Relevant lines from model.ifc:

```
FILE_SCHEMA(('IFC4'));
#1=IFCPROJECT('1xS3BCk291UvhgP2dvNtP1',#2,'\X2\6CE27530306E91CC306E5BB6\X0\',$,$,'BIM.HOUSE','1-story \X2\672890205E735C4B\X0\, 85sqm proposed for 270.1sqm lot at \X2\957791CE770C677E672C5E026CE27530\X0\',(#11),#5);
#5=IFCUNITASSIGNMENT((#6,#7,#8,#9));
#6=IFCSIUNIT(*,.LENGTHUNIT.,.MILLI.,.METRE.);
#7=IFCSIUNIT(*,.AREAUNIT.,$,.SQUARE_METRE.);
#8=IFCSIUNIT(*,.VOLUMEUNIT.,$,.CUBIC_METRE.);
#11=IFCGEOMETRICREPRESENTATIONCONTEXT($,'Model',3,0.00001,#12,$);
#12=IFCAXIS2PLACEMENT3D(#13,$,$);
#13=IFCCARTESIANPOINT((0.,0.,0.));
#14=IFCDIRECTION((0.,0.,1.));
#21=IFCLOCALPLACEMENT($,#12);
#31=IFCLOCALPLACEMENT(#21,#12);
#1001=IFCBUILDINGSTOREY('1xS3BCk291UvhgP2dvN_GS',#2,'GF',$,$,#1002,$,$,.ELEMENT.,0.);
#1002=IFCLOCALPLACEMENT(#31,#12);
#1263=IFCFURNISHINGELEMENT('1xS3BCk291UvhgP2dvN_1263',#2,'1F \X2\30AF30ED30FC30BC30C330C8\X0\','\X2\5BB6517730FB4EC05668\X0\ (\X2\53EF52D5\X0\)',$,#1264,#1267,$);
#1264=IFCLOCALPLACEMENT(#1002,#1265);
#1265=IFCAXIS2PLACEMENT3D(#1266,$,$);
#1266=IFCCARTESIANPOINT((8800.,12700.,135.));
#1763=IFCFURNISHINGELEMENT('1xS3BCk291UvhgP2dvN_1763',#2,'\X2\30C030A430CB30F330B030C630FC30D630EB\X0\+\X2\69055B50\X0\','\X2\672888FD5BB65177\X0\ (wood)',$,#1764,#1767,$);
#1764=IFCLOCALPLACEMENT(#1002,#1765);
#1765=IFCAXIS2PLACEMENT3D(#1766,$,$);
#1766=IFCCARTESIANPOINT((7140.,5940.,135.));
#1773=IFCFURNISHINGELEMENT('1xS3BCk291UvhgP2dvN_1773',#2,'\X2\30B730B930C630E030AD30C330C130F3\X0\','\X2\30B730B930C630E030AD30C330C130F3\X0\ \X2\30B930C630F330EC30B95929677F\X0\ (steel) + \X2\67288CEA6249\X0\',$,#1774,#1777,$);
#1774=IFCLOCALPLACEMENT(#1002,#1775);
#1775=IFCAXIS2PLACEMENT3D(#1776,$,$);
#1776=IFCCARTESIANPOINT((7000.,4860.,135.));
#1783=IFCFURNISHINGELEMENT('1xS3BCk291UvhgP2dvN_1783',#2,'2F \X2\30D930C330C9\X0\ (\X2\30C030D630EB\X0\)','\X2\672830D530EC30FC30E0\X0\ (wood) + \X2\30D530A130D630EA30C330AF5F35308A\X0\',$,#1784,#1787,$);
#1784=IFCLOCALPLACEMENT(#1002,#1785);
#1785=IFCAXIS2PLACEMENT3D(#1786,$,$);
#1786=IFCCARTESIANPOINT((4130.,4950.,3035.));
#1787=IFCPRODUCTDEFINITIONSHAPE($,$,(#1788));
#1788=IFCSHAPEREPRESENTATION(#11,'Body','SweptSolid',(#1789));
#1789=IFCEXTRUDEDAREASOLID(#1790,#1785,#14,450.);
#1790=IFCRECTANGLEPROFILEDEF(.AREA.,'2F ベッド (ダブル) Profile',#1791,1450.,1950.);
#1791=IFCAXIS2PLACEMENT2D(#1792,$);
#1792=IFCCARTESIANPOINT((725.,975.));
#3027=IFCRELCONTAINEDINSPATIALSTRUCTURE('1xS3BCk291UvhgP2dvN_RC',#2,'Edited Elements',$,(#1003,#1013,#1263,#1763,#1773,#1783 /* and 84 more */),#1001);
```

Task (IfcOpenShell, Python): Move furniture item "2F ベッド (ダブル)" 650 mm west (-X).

```python
import ifcopenshell
import ifcopenshell.api.geometry
import ifcopenshell.util.placement
import ifcopenshell.util.unit

model = ifcopenshell.open("model.ifc")
unit_scale = ifcopenshell.util.unit.calculate_unit_scale(model)

item = model.by_id(1783)
matrix = ifcopenshell.util.placement.get_local_placement(item.ObjectPlacement)
matrix[0, 3] -= 0.65 / unit_scale
ifcopenshell.api.geometry.edit_object_placement(model, product=item, matrix=matrix, is_si=False)

print(ifcopenshell.util.placement.get_local_placement(item.ObjectPlacement).round(3) + 0.0)

model.write("model_v2.ifc")
```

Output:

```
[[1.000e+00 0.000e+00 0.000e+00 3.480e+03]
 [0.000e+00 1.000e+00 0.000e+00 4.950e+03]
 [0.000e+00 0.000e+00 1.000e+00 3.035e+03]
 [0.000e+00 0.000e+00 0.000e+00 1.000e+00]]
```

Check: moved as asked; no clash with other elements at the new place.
